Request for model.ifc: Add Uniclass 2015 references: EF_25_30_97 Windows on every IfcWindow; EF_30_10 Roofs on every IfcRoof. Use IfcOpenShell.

First a look at what the model holds.

```python
import ifcopenshell

model = ifcopenshell.open("model.ifc")
print(model.schema)
print("classifications:", [c.Name for c in model.by_type("IfcClassification")])
for ifc_class in ("IfcDoor", "IfcRoof", "IfcStair", "IfcWall", "IfcWindow"):
    print(ifc_class, len(model.by_type(ifc_class)))
```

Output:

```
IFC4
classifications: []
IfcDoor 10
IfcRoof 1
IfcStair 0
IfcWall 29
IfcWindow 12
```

```python
import ifcopenshell
import ifcopenshell.api.classification

model = ifcopenshell.open("model.ifc")

system = ifcopenshell.api.classification.add_classification(model, classification="Uniclass 2015")

codes = {
    "IfcWindow": ("EF_25_30_97", "Windows"),
    "IfcRoof": ("EF_30_10", "Roofs"),
}
for ifc_class, (code, name) in codes.items():
    products = model.by_type(ifc_class)
    ifcopenshell.api.classification.add_reference(
        model, products=products, classification=system, identification=code, name=name
    )
    print(code, len(products))

model.write("model_v2.ifc")
```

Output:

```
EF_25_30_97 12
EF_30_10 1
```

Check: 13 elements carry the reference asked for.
